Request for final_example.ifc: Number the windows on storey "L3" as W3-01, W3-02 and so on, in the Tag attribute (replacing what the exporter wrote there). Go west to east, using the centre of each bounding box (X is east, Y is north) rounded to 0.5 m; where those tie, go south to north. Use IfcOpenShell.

First a look at what the model holds.

```python
import ifcopenshell
import ifcopenshell.util.element
import ifcopenshell.util.placement

model = ifcopenshell.open("final_example.ifc")
print(model.schema)
storey = next(s for s in model.by_type("IfcBuildingStorey") if s.Name == "L3")
windows = [e for e in ifcopenshell.util.element.get_decomposition(storey) if e.is_a("IfcWindow")]
for e in sorted(windows, key=lambda e: e.id()):
    origin = ifcopenshell.util.placement.get_local_placement(e.ObjectPlacement)[:3, 3]
    print(e.id(), e.Tag, e.Name, origin.round(2) + 0.0, sep=" | ")
```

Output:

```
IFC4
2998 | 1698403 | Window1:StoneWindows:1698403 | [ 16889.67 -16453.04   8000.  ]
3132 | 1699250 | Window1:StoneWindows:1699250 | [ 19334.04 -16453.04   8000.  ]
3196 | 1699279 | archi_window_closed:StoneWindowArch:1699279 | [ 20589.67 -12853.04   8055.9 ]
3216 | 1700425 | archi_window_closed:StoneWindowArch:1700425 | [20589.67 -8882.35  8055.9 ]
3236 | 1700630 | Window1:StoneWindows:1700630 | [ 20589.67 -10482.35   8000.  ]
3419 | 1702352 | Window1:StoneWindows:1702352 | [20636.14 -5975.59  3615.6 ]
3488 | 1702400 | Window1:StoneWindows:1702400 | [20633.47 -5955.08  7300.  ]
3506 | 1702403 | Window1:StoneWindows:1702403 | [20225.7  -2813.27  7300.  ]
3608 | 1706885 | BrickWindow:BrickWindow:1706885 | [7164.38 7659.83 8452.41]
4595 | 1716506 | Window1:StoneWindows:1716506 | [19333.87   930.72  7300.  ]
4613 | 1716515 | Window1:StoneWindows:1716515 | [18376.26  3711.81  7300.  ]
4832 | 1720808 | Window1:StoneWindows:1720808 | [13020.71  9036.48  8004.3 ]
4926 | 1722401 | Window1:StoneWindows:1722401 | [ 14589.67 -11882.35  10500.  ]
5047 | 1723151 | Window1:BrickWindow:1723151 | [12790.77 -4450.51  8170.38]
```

```python
import ifcopenshell
import ifcopenshell.geom
import ifcopenshell.util.element
import ifcopenshell.util.shape

model = ifcopenshell.open("final_example.ifc")
settings = ifcopenshell.geom.settings()
settings.set("use-world-coords", True)


def centre(element):
    shape = ifcopenshell.geom.create_shape(settings, element)
    return ifcopenshell.util.shape.get_bbox_centroid(shape.geometry)


storey = next(s for s in model.by_type("IfcBuildingStorey") if s.Name == "L3")
windows = [e for e in ifcopenshell.util.element.get_decomposition(storey) if e.is_a("IfcWindow")]

# Insertion points can sit at a corner or the storey origin, so sort by the geometry (in metres).
centres = {e: centre(e) for e in windows}
windows.sort(key=lambda e: (round(centres[e][0] / 0.5), centres[e][1]))

for i, e in enumerate(windows, start=1):
    number = f"W3-{i:02d}"
    e.Tag = number
    print(e.id(), number)

model.write("final_example_updated.ifc")
```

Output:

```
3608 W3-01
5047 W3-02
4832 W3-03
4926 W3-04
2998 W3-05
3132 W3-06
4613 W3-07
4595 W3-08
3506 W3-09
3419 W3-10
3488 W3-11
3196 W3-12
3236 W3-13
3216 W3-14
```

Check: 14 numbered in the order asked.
